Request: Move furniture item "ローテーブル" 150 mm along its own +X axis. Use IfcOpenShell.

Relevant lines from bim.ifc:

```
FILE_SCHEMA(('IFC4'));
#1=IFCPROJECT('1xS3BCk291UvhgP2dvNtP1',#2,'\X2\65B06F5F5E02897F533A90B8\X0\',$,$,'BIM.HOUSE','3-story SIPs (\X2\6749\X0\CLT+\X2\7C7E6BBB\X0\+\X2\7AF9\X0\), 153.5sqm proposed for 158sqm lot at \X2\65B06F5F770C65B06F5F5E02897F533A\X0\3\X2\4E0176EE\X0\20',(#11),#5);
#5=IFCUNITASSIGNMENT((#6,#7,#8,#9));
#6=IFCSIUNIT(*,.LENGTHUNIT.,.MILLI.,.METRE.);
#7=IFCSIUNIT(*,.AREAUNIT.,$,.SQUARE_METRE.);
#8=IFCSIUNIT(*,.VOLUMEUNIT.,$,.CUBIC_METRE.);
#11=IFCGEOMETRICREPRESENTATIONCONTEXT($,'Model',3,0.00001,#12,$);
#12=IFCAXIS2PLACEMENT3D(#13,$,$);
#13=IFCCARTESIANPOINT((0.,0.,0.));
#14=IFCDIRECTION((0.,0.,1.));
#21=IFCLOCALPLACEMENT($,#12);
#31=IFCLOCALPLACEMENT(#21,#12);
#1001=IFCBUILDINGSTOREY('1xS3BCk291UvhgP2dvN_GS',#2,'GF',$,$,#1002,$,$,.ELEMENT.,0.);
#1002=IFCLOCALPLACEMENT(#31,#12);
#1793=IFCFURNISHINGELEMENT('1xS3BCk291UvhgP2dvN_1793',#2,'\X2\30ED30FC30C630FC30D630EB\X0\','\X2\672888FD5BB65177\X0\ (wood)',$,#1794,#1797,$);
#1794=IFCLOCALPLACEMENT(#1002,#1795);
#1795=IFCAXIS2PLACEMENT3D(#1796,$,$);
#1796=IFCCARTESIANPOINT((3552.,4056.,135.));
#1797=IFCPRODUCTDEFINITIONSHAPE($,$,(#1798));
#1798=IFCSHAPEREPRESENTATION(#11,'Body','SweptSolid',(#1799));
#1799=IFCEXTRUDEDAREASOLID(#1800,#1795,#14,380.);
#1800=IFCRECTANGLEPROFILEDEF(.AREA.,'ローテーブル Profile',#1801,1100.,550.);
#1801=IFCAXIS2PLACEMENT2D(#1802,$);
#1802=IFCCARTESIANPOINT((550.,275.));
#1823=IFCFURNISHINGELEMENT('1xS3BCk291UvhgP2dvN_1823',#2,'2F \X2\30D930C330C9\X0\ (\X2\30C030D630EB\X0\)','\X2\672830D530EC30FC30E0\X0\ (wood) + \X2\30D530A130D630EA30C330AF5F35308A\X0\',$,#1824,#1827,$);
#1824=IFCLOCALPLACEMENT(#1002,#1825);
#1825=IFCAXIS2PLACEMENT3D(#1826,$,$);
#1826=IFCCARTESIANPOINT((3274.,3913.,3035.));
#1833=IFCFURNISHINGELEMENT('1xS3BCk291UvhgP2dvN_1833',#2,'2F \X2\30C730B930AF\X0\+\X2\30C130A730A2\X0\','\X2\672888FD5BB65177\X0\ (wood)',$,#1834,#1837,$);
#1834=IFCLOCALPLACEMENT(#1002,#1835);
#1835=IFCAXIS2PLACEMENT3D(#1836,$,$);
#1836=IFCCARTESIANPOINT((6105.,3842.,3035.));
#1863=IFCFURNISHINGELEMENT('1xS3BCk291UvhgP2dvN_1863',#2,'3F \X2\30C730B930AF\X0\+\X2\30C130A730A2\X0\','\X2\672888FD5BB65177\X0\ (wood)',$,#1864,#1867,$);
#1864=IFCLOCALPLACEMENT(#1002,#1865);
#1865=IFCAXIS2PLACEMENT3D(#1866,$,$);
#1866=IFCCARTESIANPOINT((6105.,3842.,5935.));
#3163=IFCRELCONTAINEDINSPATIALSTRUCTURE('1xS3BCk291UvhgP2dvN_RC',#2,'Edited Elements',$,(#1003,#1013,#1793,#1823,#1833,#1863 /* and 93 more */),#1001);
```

```python
import ifcopenshell
import ifcopenshell.api.geometry
import ifcopenshell.util.placement
import ifcopenshell.util.unit

model = ifcopenshell.open("bim.ifc")
unit_scale = ifcopenshell.util.unit.calculate_unit_scale(model)

item = model.by_guid("1xS3BCk291UvhgP2dvN_1793")
matrix = ifcopenshell.util.placement.get_local_placement(item.ObjectPlacement)
matrix[:3, 3] += matrix[:3, 0] * 0.15 / unit_scale
ifcopenshell.api.geometry.edit_object_placement(model, product=item, matrix=matrix, is_si=False)

print(ifcopenshell.util.placement.get_local_placement(item.ObjectPlacement).round(3) + 0.0)

model.write("bim_v2.ifc")
```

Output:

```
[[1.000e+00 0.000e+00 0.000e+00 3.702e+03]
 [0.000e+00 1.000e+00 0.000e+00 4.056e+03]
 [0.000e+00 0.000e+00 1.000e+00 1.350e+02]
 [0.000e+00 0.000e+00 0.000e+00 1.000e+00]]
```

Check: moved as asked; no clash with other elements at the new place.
